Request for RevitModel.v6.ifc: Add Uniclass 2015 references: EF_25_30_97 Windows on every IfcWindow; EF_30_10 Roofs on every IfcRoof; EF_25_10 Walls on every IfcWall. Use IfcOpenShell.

First a look at what the model holds.

```python
import ifcopenshell

model = ifcopenshell.open("RevitModel.v6.ifc")
print(model.schema)
print("classifications:", [c.Name for c in model.by_type("IfcClassification")])
for ifc_class in ("IfcDoor", "IfcRoof", "IfcStair", "IfcWall", "IfcWindow"):
    print(ifc_class, len(model.by_type(ifc_class)))
```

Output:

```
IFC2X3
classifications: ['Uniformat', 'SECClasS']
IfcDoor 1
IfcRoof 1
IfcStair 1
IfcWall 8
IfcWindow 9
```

```python
import ifcopenshell
import ifcopenshell.api.classification

model = ifcopenshell.open("RevitModel.v6.ifc")

# IFC2X3 requires Source and Edition and has no link from the project to the system.
system = model.create_entity("IfcClassification", Source="NBS", Edition="2015", Name="Uniclass 2015")

codes = {
    "IfcWindow": ("EF_25_30_97", "Windows"),
    "IfcRoof": ("EF_30_10", "Roofs"),
    "IfcWall": ("EF_25_10", "Walls"),
}
for ifc_class, (code, name) in codes.items():
    products = model.by_type(ifc_class)
    ifcopenshell.api.classification.add_reference(
        model, products=products, classification=system, identification=code, name=name
    )
    print(code, len(products))

model.write("RevitModel.v6_updated.ifc")
```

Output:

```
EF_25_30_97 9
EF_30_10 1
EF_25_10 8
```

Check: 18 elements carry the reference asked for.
